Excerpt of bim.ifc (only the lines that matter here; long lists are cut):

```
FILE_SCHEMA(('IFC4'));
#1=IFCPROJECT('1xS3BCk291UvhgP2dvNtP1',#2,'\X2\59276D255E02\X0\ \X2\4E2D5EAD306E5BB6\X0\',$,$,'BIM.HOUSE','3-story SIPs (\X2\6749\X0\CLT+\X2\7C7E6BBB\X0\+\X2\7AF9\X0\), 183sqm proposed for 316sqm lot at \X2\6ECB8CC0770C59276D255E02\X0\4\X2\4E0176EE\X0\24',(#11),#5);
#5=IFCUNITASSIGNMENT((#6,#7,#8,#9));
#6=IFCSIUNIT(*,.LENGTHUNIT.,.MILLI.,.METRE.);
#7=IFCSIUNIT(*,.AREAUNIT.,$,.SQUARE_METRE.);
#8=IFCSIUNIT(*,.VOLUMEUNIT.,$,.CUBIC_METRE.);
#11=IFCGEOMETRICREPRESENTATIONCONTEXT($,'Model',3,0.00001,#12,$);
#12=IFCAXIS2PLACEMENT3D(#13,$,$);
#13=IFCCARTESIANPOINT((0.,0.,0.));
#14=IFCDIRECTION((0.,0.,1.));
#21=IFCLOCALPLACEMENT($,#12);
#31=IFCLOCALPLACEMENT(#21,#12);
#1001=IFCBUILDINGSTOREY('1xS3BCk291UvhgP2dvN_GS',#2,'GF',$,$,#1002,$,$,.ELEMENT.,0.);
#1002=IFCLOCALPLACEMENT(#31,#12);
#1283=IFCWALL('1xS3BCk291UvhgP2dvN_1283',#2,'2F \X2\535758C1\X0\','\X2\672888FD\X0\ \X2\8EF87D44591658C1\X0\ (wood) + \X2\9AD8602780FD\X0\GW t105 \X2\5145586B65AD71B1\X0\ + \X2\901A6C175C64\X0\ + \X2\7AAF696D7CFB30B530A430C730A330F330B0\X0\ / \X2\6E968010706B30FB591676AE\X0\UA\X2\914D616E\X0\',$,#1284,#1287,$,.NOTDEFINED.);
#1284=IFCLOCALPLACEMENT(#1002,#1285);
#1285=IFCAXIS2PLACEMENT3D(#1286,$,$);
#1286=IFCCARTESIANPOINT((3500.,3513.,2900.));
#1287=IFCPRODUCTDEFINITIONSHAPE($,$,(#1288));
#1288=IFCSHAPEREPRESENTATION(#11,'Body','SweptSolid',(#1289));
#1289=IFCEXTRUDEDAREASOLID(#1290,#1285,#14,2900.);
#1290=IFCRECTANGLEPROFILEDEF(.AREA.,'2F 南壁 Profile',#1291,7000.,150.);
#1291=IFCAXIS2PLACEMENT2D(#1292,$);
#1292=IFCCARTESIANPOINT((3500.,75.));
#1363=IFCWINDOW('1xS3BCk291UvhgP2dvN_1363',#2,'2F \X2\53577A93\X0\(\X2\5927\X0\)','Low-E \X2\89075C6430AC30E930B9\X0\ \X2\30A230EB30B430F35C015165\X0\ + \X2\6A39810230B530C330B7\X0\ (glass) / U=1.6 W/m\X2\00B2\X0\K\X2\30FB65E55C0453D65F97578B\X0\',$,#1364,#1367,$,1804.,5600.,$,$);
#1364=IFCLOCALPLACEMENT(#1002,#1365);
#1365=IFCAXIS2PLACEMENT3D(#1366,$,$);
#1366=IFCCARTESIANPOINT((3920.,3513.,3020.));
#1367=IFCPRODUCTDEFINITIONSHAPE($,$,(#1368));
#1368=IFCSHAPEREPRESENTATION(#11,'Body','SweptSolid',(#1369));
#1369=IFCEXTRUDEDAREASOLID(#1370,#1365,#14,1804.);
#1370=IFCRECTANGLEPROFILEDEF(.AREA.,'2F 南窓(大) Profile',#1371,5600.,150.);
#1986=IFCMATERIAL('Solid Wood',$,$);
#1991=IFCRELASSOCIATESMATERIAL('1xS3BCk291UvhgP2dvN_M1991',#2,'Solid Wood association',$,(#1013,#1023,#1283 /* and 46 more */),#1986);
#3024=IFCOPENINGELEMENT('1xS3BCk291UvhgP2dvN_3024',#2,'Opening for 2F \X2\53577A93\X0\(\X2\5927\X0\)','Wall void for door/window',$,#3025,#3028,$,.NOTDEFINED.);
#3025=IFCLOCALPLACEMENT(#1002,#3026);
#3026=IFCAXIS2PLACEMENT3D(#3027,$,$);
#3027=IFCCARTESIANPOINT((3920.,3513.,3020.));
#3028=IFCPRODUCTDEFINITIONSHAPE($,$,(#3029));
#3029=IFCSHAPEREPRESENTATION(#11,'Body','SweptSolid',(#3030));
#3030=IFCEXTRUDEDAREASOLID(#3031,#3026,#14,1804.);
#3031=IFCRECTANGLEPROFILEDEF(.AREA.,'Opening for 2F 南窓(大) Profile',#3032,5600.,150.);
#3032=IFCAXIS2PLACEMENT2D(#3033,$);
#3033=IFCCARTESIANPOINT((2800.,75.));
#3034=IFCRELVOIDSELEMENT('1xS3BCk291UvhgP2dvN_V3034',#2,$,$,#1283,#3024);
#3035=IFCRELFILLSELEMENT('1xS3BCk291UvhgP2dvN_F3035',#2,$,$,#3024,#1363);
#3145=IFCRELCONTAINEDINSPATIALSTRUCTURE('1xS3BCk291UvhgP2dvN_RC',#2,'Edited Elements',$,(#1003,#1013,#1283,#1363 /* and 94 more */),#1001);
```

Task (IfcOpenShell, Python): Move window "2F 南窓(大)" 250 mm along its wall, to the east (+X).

```python
import ifcopenshell
import ifcopenshell.api.geometry
import ifcopenshell.util.placement

model = ifcopenshell.open("bim.ifc")

window = model.by_guid("1xS3BCk291UvhgP2dvN_1363")
opening = window.FillsVoids[0].RelatingOpeningElement
wall = opening.VoidsElements[0].RelatingBuildingElement

wall_matrix = ifcopenshell.util.placement.get_local_placement(wall.ObjectPlacement)
shift = wall_matrix[:3, 0] * 250.0
before = ifcopenshell.util.placement.get_local_placement(window.ObjectPlacement)[:3, 3].copy()

# The window is not placed relative to its opening, so move both.
for product in (opening, window):
    matrix = ifcopenshell.util.placement.get_local_placement(product.ObjectPlacement)
    matrix[:3, 3] += shift
    ifcopenshell.api.geometry.edit_object_placement(model, product=product, matrix=matrix, is_si=False)

after = ifcopenshell.util.placement.get_local_placement(window.ObjectPlacement)[:3, 3]
print("window moved by", (after - before).round(3) + 0.0)

model.write("bim_v2.ifc")
```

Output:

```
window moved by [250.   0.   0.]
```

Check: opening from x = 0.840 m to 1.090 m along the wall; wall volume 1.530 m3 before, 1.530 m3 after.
